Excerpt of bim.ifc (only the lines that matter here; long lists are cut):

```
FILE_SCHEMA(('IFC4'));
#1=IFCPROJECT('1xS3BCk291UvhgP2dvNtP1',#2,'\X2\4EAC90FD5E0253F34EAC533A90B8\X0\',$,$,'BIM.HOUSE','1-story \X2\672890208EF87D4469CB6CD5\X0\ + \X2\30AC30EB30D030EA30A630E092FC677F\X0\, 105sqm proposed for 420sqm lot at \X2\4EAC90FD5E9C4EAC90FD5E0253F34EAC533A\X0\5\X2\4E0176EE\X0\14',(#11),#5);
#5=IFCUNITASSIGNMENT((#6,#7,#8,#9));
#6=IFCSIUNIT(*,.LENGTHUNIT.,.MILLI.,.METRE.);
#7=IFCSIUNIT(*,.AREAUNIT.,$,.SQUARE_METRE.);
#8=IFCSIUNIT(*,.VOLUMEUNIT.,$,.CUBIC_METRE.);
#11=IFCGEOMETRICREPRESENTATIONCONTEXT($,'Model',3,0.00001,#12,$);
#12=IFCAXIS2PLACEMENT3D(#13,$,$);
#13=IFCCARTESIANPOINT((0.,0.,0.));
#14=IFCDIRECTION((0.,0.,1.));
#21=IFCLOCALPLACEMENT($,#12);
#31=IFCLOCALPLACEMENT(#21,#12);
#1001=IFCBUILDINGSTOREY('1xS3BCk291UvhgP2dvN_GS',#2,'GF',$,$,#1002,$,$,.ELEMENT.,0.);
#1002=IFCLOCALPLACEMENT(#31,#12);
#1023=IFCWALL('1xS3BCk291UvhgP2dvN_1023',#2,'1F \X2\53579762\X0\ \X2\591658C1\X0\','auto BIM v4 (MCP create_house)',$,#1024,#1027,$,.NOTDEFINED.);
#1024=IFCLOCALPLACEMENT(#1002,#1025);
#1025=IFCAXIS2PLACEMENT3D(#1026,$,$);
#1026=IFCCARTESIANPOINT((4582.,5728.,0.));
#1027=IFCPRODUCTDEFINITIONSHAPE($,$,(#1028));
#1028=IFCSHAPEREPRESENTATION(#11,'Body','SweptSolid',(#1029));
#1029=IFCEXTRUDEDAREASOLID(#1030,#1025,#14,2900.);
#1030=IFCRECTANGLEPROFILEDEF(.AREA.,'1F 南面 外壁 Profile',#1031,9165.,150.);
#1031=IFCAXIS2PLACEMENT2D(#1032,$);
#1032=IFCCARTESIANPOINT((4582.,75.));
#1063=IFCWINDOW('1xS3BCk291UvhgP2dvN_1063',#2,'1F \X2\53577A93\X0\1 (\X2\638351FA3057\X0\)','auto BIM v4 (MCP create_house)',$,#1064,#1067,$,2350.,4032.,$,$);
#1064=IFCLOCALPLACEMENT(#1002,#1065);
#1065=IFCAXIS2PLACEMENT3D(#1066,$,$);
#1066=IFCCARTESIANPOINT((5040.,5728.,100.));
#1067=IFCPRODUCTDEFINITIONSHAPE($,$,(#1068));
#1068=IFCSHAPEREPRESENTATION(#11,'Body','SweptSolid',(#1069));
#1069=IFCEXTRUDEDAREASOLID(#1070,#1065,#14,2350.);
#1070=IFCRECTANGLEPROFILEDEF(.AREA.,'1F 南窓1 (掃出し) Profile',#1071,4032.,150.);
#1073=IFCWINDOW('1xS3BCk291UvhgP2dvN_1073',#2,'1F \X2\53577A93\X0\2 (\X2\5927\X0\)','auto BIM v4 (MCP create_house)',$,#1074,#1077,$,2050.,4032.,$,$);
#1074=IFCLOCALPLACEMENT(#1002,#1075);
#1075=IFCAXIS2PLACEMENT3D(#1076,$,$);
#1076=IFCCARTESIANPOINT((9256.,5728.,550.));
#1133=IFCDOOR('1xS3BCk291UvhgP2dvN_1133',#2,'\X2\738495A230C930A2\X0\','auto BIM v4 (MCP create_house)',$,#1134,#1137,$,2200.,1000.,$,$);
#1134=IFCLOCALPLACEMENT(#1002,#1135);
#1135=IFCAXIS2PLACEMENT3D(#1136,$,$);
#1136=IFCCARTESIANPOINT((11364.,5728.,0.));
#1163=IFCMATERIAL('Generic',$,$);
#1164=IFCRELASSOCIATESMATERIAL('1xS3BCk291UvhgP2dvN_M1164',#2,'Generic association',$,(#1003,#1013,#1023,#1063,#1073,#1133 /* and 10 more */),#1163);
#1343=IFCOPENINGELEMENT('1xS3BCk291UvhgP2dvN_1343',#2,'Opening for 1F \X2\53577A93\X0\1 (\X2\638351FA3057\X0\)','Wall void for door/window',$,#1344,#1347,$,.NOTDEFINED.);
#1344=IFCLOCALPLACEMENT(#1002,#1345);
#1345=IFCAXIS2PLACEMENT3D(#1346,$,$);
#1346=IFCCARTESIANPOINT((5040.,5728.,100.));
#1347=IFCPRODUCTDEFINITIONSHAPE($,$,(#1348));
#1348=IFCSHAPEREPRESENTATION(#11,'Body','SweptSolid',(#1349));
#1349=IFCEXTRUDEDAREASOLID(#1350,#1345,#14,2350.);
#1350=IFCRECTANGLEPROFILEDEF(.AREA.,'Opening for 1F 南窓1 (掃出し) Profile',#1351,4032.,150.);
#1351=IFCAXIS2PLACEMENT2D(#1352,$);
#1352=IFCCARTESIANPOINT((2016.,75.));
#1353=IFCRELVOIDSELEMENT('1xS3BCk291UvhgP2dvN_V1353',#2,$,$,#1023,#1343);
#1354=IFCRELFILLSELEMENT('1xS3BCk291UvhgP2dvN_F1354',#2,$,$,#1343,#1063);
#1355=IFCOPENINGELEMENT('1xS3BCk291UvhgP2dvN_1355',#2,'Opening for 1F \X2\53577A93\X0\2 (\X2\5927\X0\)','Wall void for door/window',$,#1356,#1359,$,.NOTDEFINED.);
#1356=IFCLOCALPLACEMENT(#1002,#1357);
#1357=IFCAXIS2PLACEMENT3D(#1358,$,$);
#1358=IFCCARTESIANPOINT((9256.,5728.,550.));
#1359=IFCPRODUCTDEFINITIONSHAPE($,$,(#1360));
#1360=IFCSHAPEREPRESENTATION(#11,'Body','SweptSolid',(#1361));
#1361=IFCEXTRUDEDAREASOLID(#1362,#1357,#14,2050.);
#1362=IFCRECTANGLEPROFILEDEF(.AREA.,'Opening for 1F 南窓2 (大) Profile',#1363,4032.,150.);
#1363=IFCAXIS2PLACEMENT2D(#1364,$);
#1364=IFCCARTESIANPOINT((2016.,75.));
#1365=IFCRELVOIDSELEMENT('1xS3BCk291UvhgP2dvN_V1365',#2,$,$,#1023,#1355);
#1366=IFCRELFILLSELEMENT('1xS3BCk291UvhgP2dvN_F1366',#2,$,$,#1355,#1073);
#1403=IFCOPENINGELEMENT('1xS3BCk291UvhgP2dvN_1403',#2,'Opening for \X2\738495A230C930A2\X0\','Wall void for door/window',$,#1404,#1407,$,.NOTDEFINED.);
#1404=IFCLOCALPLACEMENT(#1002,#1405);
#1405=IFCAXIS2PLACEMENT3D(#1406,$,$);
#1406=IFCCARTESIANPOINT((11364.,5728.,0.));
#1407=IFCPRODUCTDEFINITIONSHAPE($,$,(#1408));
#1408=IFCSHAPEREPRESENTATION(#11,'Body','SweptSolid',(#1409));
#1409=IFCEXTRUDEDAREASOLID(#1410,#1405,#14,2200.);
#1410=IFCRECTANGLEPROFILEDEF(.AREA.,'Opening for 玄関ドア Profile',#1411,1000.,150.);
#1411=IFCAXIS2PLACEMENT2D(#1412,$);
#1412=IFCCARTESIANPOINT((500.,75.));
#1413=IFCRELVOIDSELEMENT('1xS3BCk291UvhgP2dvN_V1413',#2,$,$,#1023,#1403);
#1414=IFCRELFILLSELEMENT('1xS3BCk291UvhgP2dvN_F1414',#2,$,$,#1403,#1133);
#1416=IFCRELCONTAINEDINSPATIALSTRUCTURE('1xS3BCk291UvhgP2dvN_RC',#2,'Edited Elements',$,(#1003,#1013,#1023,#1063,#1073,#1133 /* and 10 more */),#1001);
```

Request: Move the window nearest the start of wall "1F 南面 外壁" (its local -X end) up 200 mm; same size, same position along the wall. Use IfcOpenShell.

```python
import numpy as np
import ifcopenshell
import ifcopenshell.api.geometry
import ifcopenshell.util.placement
import ifcopenshell.util.unit

model = ifcopenshell.open("bim.ifc")
unit_scale = ifcopenshell.util.unit.calculate_unit_scale(model)

window = model.by_guid("1xS3BCk291UvhgP2dvN_1063")
opening = window.FillsVoids[0].RelatingOpeningElement
dz = 200.0

shift = np.array([0.0, 0.0, dz])
# The window is not placed relative to its opening, so move both.
for product in (opening, window):
    matrix = ifcopenshell.util.placement.get_local_placement(product.ObjectPlacement)
    matrix[:3, 3] += shift
    ifcopenshell.api.geometry.edit_object_placement(model, product=product, matrix=matrix, is_si=False)

print(f"moved by {dz * unit_scale:+.3f} m")

model.write("bim_rev.ifc")
```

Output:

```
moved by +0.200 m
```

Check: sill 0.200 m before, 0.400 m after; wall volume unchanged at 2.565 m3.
